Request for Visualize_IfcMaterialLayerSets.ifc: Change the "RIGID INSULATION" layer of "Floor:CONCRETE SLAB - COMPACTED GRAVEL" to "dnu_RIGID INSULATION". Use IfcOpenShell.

First a look at what the model holds.

```python
import ifcopenshell
import ifcopenshell.util.element

model = ifcopenshell.open("Visualize_IfcMaterialLayerSets.ifc")
print(model.schema)
for layer_set in model.by_type("IfcMaterialLayerSet"):
    if layer_set.LayerSetName == "Floor:CONCRETE SLAB - COMPACTED GRAVEL":
        for layer in layer_set.MaterialLayers:
            print(layer.id(), layer.Material and layer.Material.Name, layer.LayerThickness, sep=" | ")
        print(len(ifcopenshell.util.element.get_elements_by_material(model, layer_set)), "elements and types use it")
print(sorted(m.Name for m in model.by_type("IfcMaterial") if m.Name)[:60])
```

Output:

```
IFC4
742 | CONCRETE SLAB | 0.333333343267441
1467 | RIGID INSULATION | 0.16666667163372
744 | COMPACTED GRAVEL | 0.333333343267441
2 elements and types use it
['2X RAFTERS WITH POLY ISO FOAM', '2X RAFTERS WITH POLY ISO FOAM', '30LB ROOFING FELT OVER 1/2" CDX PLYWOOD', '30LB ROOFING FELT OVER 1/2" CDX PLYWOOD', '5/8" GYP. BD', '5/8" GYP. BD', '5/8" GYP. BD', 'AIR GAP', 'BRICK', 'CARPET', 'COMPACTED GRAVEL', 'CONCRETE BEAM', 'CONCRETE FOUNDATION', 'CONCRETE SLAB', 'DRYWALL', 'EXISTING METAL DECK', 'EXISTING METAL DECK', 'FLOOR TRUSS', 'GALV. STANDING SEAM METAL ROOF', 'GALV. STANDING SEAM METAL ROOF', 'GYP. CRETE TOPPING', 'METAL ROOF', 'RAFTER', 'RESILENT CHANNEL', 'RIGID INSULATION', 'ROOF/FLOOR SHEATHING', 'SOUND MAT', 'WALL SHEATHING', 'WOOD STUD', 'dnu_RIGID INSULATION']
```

```python
import ifcopenshell
import ifcopenshell.api.material

model = ifcopenshell.open("Visualize_IfcMaterialLayerSets.ifc")

layer_set = next(s for s in model.by_type("IfcMaterialLayerSet") if s.LayerSetName == "Floor:CONCRETE SLAB - COMPACTED GRAVEL")
layer = next(l for l in layer_set.MaterialLayers if l.Material and l.Material.Name == "RIGID INSULATION")
material = next(m for m in model.by_type("IfcMaterial") if m.Name == "dnu_RIGID INSULATION")

# Point this one layer at the other material; renaming the old one would change it everywhere.
ifcopenshell.api.material.edit_layer(model, layer=layer, attributes={}, material=material)

print([l.Material.Name if l.Material else None for l in layer_set.MaterialLayers])

model.write("Visualize_IfcMaterialLayerSets_v2.ifc")
```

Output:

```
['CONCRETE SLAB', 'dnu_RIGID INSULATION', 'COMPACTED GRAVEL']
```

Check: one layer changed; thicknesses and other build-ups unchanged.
